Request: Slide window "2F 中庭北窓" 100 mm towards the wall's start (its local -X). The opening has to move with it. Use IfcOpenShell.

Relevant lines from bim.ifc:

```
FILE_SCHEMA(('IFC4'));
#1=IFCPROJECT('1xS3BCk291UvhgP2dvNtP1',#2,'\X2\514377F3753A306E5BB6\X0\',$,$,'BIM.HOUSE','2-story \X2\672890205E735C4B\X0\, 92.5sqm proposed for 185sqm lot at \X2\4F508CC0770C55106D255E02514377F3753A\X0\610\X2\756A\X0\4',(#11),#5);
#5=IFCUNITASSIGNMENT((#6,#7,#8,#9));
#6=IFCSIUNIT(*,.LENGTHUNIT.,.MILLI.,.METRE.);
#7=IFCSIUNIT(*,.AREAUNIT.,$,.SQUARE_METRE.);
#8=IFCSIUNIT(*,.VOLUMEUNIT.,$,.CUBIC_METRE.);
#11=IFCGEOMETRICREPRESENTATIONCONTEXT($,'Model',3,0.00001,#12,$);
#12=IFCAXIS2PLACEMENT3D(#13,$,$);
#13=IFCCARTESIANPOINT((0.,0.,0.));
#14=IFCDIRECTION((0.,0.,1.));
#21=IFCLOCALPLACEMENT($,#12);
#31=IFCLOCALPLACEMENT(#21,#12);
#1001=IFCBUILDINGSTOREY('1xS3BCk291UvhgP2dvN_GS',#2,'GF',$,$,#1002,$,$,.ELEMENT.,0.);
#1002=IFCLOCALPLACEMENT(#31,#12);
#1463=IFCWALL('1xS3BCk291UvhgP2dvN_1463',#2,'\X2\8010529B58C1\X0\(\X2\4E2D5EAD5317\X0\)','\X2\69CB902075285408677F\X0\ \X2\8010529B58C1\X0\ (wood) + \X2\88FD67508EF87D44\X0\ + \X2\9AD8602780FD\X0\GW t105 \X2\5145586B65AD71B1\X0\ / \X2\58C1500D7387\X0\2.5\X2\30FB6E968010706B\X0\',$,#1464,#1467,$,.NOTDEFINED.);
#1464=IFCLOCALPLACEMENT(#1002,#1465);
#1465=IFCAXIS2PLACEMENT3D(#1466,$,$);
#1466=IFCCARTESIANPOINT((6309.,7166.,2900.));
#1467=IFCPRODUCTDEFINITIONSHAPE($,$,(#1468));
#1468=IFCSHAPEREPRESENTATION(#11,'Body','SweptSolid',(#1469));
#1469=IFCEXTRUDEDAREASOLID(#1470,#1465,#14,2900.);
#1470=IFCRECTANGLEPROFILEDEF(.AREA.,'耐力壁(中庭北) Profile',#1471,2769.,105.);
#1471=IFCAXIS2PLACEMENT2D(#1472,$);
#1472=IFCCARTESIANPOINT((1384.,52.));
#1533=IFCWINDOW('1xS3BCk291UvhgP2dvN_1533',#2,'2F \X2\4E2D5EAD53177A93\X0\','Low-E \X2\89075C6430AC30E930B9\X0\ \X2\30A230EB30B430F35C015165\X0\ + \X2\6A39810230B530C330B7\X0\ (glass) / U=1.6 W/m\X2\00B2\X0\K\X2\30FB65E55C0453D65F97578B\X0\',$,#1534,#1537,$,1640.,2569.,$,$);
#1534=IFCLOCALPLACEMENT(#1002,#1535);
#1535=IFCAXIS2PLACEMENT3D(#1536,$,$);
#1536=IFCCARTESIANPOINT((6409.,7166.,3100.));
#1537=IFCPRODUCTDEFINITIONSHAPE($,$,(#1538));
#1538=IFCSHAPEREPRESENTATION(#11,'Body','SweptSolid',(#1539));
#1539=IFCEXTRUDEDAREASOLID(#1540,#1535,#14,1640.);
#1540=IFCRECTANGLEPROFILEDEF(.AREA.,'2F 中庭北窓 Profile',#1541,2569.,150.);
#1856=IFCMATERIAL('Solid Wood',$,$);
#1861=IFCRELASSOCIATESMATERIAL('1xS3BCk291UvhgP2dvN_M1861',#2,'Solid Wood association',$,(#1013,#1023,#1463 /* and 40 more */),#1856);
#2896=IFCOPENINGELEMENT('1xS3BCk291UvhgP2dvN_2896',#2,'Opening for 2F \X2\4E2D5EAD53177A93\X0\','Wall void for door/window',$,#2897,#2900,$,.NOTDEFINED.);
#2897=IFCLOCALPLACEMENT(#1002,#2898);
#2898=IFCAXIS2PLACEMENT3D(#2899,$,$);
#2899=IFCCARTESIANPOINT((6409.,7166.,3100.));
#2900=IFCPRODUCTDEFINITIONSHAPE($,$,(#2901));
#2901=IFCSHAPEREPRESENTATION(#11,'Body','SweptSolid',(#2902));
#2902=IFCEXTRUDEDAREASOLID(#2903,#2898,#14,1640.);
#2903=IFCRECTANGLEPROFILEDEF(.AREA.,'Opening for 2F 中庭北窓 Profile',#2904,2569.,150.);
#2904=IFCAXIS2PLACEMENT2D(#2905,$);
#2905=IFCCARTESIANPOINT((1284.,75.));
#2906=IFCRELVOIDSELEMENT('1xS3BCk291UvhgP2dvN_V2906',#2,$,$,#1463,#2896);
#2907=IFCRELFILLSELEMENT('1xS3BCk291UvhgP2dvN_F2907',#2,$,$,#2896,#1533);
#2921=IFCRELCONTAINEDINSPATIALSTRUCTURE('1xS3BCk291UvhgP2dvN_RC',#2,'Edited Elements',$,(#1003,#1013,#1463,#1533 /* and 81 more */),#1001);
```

```python
import ifcopenshell
import ifcopenshell.api.geometry
import ifcopenshell.util.placement

model = ifcopenshell.open("bim.ifc")

window = model.by_guid("1xS3BCk291UvhgP2dvN_1533")
opening = window.FillsVoids[0].RelatingOpeningElement
wall = opening.VoidsElements[0].RelatingBuildingElement

wall_matrix = ifcopenshell.util.placement.get_local_placement(wall.ObjectPlacement)
shift = wall_matrix[:3, 0] * -100.0
before = ifcopenshell.util.placement.get_local_placement(window.ObjectPlacement)[:3, 3].copy()

# The window is not placed relative to its opening, so move both.
for product in (opening, window):
    matrix = ifcopenshell.util.placement.get_local_placement(product.ObjectPlacement)
    matrix[:3, 3] += shift
    ifcopenshell.api.geometry.edit_object_placement(model, product=product, matrix=matrix, is_si=False)

after = ifcopenshell.util.placement.get_local_placement(window.ObjectPlacement)[:3, 3]
print("window moved by", (after - before).round(3) + 0.0)

model.write("bim_rev.ifc")
```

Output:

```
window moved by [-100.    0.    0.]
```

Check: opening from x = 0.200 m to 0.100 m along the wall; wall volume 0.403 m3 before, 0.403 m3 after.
